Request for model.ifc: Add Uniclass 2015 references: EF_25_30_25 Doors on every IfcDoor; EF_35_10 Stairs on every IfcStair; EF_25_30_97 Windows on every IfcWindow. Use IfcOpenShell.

First a look at what the model holds.

```python
import ifcopenshell

model = ifcopenshell.open("model.ifc")
print(model.schema)
print("classifications:", [c.Name for c in model.by_type("IfcClassification")])
for ifc_class in ("IfcDoor", "IfcRoof", "IfcStair", "IfcWall", "IfcWindow"):
    print(ifc_class, len(model.by_type(ifc_class)))
```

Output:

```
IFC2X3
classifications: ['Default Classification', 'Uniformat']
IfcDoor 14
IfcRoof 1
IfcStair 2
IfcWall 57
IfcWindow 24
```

```python
import ifcopenshell
import ifcopenshell.api.classification

model = ifcopenshell.open("model.ifc")

# IFC2X3 requires Source and Edition and has no link from the project to the system.
system = model.create_entity("IfcClassification", Source="NBS", Edition="2015", Name="Uniclass 2015")

codes = {
    "IfcDoor": ("EF_25_30_25", "Doors"),
    "IfcStair": ("EF_35_10", "Stairs"),
    "IfcWindow": ("EF_25_30_97", "Windows"),
}
for ifc_class, (code, name) in codes.items():
    products = model.by_type(ifc_class)
    ifcopenshell.api.classification.add_reference(
        model, products=products, classification=system, identification=code, name=name
    )
    print(code, len(products))

model.write("model-out.ifc")
```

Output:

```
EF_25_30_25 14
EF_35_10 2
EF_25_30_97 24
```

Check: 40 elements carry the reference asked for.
